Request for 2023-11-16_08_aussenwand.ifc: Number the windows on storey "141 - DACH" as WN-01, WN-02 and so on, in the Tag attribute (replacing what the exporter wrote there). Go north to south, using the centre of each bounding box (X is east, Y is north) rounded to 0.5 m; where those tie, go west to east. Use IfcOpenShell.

First a look at what the model holds.

```python
import ifcopenshell
import ifcopenshell.util.element
import ifcopenshell.util.placement

model = ifcopenshell.open("2023-11-16_08_aussenwand.ifc")
print(model.schema)
storey = next(s for s in model.by_type("IfcBuildingStorey") if s.Name == "141 - DACH")
windows = [e for e in ifcopenshell.util.element.get_decomposition(storey) if e.is_a("IfcWindow")]
for e in sorted(windows, key=lambda e: e.id()):
    origin = ifcopenshell.util.placement.get_local_placement(e.ObjectPlacement)[:3, 3]
    print(e.id(), e.Tag, e.Name, origin.round(2) + 0.0, sep=" | ")
```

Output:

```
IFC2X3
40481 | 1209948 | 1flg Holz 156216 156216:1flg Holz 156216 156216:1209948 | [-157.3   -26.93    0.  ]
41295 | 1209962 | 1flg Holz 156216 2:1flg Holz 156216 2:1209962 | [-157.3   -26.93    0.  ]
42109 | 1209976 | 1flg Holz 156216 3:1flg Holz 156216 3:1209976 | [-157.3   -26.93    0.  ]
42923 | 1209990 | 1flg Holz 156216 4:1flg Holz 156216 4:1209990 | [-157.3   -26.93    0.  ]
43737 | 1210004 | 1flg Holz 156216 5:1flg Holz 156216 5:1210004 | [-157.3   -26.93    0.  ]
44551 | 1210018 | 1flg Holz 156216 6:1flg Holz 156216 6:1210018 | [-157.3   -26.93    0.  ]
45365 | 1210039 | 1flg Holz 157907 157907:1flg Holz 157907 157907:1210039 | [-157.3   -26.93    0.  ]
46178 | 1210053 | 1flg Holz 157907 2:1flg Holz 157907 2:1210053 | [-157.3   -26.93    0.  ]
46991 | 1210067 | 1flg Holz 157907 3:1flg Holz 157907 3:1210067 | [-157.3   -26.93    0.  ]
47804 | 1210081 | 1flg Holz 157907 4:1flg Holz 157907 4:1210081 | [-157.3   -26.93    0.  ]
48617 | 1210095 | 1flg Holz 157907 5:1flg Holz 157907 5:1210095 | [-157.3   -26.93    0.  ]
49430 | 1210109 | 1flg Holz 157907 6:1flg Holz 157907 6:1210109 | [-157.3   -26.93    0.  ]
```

```python
import ifcopenshell
import ifcopenshell.geom
import ifcopenshell.util.element
import ifcopenshell.util.shape

model = ifcopenshell.open("2023-11-16_08_aussenwand.ifc")
settings = ifcopenshell.geom.settings()
settings.set("use-world-coords", True)


def centre(element):
    shape = ifcopenshell.geom.create_shape(settings, element)
    return ifcopenshell.util.shape.get_bbox_centroid(shape.geometry)


storey = next(s for s in model.by_type("IfcBuildingStorey") if s.Name == "141 - DACH")
windows = [e for e in ifcopenshell.util.element.get_decomposition(storey) if e.is_a("IfcWindow")]

# Insertion points can sit at a corner or the storey origin, so sort by the geometry (in metres).
centres = {e: centre(e) for e in windows}
windows.sort(key=lambda e: (-round(centres[e][1] / 0.5), centres[e][0]))

for i, e in enumerate(windows, start=1):
    number = f"WN-{i:02d}"
    e.Tag = number
    print(e.id(), number)

model.write("2023-11-16_08_aussenwand_edited.ifc")
```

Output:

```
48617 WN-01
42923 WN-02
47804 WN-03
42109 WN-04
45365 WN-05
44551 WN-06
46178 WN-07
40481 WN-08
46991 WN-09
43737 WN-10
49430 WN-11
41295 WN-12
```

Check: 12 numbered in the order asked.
